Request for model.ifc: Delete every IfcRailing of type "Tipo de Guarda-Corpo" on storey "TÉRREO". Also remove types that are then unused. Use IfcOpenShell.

First a look at what the model holds.

```python
import ifcopenshell
import ifcopenshell.util.element

model = ifcopenshell.open("model.ifc")
print(model.schema)
storey = next(s for s in model.by_type("IfcBuildingStorey") if s.Name == "TÉRREO")
railings = [e for e in ifcopenshell.util.element.get_decomposition(storey) if e.is_a("IfcRailing")]
seen = {}
for e in railings:
    element_type = ifcopenshell.util.element.get_type(e)
    name = element_type.Name if element_type not in (None, e) else None
    seen[name] = seen.get(name, 0) + 1
for name, count in sorted(seen.items(), key=str):
    print(count, "x", name)
```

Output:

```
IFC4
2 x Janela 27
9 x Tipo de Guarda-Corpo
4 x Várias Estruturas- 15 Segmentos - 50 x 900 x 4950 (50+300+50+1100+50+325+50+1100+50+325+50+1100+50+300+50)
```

```python
import ifcopenshell
import ifcopenshell.api.root
import ifcopenshell.util.element

model = ifcopenshell.open("model.ifc")

storey = next(s for s in model.by_type("IfcBuildingStorey") if s.Name == "TÉRREO")
railings = [e for e in ifcopenshell.util.element.get_decomposition(storey) if e.is_a("IfcRailing")]
targets = [e for e in railings if (t := ifcopenshell.util.element.get_type(e)) not in (None, e) and t.Name == "Tipo de Guarda-Corpo"]
types = {ifcopenshell.util.element.get_type(e) for e in targets} - {None, *targets}

for e in targets:
    ifcopenshell.api.root.remove_product(model, product=e)
print(len(targets), "removed")

unused = [t for t in types if not ifcopenshell.util.element.get_types(t)]
for t in unused:
    ifcopenshell.api.root.remove_product(model, product=t)
print(len(unused), "unused types removed")

model.write("model_rev.ifc")
```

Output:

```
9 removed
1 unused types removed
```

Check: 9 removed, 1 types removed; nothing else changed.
